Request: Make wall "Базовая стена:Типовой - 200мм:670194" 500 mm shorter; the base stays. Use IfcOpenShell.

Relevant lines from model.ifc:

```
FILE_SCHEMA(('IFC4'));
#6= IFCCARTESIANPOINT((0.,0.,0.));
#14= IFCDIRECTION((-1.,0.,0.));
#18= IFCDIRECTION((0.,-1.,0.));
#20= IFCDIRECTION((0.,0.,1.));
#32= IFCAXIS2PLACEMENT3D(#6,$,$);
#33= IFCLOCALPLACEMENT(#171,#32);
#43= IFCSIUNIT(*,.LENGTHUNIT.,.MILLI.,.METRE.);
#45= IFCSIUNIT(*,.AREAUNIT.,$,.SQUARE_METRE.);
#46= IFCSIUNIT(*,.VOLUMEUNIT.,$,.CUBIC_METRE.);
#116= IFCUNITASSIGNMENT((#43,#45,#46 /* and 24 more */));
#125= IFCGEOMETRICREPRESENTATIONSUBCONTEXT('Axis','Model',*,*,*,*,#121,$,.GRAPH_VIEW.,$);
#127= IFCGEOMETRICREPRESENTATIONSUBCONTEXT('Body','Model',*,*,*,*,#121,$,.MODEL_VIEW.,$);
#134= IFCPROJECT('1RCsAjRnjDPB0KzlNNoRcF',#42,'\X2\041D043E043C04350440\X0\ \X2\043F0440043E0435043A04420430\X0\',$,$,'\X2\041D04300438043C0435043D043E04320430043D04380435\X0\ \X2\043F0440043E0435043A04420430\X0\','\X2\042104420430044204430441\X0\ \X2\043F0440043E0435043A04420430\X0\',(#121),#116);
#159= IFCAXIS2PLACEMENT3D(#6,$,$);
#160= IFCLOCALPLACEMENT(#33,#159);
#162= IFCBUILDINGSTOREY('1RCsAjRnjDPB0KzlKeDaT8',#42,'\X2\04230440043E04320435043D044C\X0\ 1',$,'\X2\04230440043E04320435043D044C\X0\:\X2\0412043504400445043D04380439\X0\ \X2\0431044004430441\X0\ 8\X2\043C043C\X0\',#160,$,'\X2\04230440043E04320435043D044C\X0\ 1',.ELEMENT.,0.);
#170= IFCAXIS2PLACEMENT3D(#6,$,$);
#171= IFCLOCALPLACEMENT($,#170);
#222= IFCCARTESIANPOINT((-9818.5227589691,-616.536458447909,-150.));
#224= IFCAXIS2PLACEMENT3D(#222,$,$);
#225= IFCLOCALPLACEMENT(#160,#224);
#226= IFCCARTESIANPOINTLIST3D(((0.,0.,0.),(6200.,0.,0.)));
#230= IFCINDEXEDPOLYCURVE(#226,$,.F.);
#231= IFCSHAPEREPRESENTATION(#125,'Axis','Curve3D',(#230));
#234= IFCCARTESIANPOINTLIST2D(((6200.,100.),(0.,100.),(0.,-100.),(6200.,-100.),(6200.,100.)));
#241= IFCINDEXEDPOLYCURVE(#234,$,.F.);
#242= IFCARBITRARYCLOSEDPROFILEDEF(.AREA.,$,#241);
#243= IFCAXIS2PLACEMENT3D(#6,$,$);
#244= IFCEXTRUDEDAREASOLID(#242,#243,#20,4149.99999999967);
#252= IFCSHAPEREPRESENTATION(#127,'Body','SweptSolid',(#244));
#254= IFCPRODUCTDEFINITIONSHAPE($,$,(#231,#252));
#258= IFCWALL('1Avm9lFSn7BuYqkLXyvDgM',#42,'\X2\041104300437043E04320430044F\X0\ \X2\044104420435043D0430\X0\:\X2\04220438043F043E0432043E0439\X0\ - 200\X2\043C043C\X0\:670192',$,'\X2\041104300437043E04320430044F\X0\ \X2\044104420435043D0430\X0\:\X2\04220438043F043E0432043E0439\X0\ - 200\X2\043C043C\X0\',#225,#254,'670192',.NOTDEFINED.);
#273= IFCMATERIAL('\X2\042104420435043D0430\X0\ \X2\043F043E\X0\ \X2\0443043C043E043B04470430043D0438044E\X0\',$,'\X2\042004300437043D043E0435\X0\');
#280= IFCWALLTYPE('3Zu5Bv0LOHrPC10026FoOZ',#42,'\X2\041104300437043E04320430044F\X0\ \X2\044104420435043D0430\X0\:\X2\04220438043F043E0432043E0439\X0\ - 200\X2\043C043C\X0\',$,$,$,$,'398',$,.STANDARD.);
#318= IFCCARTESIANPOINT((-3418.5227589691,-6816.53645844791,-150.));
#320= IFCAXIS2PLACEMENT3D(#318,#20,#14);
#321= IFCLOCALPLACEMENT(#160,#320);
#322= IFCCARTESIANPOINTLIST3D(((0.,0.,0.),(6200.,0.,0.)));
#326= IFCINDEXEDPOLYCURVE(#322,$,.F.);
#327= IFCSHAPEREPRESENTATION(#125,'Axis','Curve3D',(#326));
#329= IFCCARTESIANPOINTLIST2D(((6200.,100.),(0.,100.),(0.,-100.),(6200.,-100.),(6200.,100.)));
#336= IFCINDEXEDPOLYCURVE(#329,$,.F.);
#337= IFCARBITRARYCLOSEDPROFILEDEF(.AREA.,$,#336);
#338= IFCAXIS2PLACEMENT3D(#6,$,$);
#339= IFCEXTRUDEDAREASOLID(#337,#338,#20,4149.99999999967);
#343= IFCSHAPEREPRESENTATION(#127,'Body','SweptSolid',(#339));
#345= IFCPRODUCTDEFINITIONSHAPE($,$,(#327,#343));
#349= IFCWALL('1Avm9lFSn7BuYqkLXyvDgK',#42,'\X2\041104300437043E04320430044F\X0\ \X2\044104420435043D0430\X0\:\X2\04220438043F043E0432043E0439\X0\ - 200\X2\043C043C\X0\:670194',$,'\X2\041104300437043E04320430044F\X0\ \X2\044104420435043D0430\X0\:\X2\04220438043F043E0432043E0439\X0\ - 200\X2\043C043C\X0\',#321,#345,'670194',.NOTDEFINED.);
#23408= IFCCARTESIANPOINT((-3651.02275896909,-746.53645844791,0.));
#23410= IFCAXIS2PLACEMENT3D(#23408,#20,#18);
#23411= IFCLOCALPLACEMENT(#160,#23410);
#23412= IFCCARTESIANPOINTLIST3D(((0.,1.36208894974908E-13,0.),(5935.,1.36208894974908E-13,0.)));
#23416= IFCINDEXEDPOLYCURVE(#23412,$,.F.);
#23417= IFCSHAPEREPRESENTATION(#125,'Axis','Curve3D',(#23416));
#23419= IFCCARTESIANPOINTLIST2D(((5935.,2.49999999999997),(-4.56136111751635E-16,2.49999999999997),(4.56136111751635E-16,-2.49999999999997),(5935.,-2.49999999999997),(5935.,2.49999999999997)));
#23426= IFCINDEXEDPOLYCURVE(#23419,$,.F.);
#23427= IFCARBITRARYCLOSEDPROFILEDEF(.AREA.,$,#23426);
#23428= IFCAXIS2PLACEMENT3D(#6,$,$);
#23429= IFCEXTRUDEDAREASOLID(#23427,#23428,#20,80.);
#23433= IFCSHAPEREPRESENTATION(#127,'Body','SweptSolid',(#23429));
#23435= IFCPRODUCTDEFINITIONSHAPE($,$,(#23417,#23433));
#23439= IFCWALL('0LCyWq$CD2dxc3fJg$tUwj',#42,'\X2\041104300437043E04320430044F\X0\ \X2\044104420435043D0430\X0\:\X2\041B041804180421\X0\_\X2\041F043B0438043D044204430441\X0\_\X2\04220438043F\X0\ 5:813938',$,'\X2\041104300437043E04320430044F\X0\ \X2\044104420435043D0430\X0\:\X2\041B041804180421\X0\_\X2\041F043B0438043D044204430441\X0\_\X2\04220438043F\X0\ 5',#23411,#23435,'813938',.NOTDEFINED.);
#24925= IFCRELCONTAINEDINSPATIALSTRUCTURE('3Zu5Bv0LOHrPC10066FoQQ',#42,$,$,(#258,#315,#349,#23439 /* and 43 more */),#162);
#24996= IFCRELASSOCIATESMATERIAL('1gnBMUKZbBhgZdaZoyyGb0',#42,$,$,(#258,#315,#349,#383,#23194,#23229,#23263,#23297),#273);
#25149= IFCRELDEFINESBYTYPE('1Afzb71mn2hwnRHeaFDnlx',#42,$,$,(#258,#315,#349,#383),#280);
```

```python
import ifcopenshell
import ifcopenshell.geom
import ifcopenshell.util.representation
import ifcopenshell.util.shape
import ifcopenshell.util.unit

model = ifcopenshell.open("model.ifc")
unit_scale = ifcopenshell.util.unit.calculate_unit_scale(model)
settings = ifcopenshell.geom.settings()


def volume(element):
    """Net volume in cubic metres, openings subtracted."""
    shape = ifcopenshell.geom.create_shape(settings, element)
    return ifcopenshell.util.shape.get_volume(shape.geometry)


wall = model.by_guid("1Avm9lFSn7BuYqkLXyvDgK")
before = volume(wall)

body = ifcopenshell.util.representation.get_representation(wall, "Model", "Body")
solid = body.Items[0]
old_height = solid.Depth
solid.Depth -= 0.5 / unit_scale
after = volume(wall)

print(f"height {old_height:g} -> {solid.Depth:g}, volume {before:.3f} -> {after:.3f} m3")

model.write("model_rev.ifc")
```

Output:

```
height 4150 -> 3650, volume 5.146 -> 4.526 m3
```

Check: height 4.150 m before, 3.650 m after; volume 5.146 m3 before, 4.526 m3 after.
